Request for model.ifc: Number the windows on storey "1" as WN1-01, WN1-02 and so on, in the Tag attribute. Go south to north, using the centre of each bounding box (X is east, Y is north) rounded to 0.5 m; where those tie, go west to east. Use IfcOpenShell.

First a look at what the model holds.

```python
import ifcopenshell
import ifcopenshell.util.element
import ifcopenshell.util.placement

model = ifcopenshell.open("model.ifc")
print(model.schema)
storey = next(s for s in model.by_type("IfcBuildingStorey") if s.Name == "1")
windows = [e for e in ifcopenshell.util.element.get_decomposition(storey) if e.is_a("IfcWindow")]
for e in sorted(windows, key=lambda e: e.id()):
    origin = ifcopenshell.util.placement.get_local_placement(e.ObjectPlacement)[:3, 3]
    print(e.id(), e.Tag, e.Name, origin.round(2) + 0.0, sep=" | ")
```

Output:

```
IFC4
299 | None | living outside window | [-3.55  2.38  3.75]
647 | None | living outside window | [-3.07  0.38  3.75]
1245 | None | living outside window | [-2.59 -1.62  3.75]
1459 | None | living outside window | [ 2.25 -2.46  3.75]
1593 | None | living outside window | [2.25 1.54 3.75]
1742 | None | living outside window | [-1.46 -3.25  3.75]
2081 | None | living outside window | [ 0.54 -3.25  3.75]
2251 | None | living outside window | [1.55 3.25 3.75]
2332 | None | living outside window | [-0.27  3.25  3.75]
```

```python
import ifcopenshell
import ifcopenshell.geom
import ifcopenshell.util.element
import ifcopenshell.util.shape

model = ifcopenshell.open("model.ifc")
settings = ifcopenshell.geom.settings()
settings.set("use-world-coords", True)


def centre(element):
    shape = ifcopenshell.geom.create_shape(settings, element)
    return ifcopenshell.util.shape.get_bbox_centroid(shape.geometry)


storey = next(s for s in model.by_type("IfcBuildingStorey") if s.Name == "1")
windows = [e for e in ifcopenshell.util.element.get_decomposition(storey) if e.is_a("IfcWindow")]

# Insertion points can sit at a corner or the storey origin, so sort by the geometry (in metres).
centres = {e: centre(e) for e in windows}
windows.sort(key=lambda e: (round(centres[e][1] / 0.5), centres[e][0]))

for i, e in enumerate(windows, start=1):
    number = f"WN1-{i:02d}"
    e.Tag = number
    print(e.id(), number)

model.write("model_rev.ifc")
```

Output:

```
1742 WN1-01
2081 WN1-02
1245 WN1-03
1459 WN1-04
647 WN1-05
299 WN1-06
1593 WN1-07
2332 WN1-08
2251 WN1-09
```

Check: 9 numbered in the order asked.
